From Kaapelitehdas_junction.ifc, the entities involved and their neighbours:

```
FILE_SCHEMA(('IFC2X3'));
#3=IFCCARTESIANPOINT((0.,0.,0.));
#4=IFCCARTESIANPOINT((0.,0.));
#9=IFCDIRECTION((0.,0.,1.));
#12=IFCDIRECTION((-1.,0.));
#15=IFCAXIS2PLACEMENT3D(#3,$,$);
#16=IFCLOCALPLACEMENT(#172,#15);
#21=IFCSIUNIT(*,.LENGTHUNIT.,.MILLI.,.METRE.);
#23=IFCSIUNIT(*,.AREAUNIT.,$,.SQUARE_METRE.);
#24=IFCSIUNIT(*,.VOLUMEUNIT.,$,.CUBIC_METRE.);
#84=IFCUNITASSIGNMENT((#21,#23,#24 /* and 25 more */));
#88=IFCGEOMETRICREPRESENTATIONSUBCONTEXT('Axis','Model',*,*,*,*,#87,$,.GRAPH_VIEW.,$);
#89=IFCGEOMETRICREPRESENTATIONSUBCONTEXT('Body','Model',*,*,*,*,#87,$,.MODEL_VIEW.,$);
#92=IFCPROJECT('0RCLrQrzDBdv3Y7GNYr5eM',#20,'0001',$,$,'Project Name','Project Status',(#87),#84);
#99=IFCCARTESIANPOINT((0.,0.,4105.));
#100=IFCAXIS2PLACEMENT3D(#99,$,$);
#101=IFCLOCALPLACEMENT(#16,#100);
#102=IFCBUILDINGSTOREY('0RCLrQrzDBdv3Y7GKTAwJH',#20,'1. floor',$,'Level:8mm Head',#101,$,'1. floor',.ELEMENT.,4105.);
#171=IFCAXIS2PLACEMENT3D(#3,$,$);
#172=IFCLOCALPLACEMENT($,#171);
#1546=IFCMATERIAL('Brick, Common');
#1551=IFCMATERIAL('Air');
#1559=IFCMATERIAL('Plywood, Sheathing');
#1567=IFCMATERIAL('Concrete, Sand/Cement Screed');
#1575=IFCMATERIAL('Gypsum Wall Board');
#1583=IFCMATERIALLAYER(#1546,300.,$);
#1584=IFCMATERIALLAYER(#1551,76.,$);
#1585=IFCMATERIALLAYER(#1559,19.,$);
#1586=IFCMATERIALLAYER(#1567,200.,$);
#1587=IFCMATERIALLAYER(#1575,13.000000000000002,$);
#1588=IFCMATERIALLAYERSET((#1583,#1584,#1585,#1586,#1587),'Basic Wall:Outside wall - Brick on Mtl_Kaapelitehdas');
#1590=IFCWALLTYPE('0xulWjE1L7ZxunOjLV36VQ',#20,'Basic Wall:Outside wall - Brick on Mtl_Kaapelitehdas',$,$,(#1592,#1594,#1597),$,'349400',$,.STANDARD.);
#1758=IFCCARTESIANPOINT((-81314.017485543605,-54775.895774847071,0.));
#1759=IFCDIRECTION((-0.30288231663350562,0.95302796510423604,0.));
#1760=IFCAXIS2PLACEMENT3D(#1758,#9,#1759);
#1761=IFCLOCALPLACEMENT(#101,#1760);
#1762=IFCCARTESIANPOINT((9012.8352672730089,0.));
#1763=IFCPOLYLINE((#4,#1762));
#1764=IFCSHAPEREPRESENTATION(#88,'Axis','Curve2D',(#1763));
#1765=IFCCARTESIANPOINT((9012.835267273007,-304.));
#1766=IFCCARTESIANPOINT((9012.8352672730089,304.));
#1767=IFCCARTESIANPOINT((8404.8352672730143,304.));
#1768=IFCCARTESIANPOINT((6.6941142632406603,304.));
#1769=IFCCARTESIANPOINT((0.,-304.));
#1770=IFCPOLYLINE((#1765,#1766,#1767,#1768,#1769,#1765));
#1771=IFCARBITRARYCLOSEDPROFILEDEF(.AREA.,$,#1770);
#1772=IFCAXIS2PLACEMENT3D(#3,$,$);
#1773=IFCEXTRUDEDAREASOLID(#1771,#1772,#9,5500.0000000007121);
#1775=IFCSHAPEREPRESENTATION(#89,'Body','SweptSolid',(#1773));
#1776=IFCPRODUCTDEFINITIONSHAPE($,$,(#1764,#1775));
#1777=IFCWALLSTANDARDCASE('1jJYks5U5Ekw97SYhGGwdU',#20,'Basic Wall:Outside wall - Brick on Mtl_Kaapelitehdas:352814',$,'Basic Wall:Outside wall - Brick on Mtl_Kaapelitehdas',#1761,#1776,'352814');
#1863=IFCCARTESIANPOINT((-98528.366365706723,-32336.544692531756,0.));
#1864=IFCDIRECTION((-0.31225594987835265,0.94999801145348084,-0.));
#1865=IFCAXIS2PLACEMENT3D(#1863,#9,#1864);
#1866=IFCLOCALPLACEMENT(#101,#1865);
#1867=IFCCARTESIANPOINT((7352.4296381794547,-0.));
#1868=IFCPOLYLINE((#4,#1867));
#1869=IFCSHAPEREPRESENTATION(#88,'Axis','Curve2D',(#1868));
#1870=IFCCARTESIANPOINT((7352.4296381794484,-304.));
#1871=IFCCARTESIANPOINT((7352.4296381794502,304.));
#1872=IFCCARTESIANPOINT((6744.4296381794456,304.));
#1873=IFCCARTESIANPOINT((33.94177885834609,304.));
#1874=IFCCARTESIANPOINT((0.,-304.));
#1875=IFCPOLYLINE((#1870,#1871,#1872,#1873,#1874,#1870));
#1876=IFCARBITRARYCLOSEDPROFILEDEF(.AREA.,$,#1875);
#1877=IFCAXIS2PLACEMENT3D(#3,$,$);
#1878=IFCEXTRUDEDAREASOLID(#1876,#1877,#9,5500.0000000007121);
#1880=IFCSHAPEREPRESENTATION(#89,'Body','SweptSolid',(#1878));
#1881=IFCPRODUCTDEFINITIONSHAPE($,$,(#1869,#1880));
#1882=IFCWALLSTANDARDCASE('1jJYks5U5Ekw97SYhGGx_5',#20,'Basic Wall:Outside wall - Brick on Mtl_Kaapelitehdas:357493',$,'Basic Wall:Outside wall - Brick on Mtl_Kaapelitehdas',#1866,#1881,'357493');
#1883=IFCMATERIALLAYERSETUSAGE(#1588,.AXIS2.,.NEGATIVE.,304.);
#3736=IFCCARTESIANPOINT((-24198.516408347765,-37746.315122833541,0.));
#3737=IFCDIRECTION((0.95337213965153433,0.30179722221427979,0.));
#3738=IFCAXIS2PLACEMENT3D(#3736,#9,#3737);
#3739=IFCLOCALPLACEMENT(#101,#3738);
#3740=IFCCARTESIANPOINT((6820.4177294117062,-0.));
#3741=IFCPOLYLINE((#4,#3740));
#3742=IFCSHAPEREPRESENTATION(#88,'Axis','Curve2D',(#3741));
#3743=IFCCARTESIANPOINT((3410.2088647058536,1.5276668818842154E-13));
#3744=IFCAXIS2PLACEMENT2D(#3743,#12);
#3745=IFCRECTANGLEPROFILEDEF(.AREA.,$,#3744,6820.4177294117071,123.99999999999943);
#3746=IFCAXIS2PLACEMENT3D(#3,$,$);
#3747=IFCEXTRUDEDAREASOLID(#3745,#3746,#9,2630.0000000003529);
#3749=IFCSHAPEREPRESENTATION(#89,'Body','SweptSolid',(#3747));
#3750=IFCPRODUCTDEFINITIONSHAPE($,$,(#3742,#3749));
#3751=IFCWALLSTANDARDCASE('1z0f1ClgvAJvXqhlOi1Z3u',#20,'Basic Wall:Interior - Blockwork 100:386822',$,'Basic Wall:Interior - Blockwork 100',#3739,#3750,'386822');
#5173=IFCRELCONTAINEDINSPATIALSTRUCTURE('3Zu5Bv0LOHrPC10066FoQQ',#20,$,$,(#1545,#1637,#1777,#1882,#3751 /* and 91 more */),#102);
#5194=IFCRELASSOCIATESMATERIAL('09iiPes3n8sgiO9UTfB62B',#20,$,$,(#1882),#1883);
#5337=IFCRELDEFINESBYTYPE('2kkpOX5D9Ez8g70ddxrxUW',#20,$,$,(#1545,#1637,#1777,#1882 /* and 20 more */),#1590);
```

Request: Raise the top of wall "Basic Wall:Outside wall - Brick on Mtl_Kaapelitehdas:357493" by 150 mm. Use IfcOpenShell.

```python
import ifcopenshell
import ifcopenshell.geom
import ifcopenshell.util.representation
import ifcopenshell.util.shape
import ifcopenshell.util.unit

model = ifcopenshell.open("Kaapelitehdas_junction.ifc")
unit_scale = ifcopenshell.util.unit.calculate_unit_scale(model)
settings = ifcopenshell.geom.settings()


def volume(element):
    """Net volume in cubic metres, openings subtracted."""
    shape = ifcopenshell.geom.create_shape(settings, element)
    return ifcopenshell.util.shape.get_volume(shape.geometry)


wall = model.by_guid("1jJYks5U5Ekw97SYhGGx_5")
before = volume(wall)

body = ifcopenshell.util.representation.get_representation(wall, "Model", "Body")
solid = body.Items[0]
old_height = solid.Depth
solid.Depth += 0.15 / unit_scale
after = volume(wall)

print(f"height {old_height:g} -> {solid.Depth:g}, volume {before:.3f} -> {after:.3f} m3")

model.write("Kaapelitehdas_junction_v2.ifc")
```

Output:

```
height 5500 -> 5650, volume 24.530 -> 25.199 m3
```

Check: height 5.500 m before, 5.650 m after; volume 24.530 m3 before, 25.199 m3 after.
